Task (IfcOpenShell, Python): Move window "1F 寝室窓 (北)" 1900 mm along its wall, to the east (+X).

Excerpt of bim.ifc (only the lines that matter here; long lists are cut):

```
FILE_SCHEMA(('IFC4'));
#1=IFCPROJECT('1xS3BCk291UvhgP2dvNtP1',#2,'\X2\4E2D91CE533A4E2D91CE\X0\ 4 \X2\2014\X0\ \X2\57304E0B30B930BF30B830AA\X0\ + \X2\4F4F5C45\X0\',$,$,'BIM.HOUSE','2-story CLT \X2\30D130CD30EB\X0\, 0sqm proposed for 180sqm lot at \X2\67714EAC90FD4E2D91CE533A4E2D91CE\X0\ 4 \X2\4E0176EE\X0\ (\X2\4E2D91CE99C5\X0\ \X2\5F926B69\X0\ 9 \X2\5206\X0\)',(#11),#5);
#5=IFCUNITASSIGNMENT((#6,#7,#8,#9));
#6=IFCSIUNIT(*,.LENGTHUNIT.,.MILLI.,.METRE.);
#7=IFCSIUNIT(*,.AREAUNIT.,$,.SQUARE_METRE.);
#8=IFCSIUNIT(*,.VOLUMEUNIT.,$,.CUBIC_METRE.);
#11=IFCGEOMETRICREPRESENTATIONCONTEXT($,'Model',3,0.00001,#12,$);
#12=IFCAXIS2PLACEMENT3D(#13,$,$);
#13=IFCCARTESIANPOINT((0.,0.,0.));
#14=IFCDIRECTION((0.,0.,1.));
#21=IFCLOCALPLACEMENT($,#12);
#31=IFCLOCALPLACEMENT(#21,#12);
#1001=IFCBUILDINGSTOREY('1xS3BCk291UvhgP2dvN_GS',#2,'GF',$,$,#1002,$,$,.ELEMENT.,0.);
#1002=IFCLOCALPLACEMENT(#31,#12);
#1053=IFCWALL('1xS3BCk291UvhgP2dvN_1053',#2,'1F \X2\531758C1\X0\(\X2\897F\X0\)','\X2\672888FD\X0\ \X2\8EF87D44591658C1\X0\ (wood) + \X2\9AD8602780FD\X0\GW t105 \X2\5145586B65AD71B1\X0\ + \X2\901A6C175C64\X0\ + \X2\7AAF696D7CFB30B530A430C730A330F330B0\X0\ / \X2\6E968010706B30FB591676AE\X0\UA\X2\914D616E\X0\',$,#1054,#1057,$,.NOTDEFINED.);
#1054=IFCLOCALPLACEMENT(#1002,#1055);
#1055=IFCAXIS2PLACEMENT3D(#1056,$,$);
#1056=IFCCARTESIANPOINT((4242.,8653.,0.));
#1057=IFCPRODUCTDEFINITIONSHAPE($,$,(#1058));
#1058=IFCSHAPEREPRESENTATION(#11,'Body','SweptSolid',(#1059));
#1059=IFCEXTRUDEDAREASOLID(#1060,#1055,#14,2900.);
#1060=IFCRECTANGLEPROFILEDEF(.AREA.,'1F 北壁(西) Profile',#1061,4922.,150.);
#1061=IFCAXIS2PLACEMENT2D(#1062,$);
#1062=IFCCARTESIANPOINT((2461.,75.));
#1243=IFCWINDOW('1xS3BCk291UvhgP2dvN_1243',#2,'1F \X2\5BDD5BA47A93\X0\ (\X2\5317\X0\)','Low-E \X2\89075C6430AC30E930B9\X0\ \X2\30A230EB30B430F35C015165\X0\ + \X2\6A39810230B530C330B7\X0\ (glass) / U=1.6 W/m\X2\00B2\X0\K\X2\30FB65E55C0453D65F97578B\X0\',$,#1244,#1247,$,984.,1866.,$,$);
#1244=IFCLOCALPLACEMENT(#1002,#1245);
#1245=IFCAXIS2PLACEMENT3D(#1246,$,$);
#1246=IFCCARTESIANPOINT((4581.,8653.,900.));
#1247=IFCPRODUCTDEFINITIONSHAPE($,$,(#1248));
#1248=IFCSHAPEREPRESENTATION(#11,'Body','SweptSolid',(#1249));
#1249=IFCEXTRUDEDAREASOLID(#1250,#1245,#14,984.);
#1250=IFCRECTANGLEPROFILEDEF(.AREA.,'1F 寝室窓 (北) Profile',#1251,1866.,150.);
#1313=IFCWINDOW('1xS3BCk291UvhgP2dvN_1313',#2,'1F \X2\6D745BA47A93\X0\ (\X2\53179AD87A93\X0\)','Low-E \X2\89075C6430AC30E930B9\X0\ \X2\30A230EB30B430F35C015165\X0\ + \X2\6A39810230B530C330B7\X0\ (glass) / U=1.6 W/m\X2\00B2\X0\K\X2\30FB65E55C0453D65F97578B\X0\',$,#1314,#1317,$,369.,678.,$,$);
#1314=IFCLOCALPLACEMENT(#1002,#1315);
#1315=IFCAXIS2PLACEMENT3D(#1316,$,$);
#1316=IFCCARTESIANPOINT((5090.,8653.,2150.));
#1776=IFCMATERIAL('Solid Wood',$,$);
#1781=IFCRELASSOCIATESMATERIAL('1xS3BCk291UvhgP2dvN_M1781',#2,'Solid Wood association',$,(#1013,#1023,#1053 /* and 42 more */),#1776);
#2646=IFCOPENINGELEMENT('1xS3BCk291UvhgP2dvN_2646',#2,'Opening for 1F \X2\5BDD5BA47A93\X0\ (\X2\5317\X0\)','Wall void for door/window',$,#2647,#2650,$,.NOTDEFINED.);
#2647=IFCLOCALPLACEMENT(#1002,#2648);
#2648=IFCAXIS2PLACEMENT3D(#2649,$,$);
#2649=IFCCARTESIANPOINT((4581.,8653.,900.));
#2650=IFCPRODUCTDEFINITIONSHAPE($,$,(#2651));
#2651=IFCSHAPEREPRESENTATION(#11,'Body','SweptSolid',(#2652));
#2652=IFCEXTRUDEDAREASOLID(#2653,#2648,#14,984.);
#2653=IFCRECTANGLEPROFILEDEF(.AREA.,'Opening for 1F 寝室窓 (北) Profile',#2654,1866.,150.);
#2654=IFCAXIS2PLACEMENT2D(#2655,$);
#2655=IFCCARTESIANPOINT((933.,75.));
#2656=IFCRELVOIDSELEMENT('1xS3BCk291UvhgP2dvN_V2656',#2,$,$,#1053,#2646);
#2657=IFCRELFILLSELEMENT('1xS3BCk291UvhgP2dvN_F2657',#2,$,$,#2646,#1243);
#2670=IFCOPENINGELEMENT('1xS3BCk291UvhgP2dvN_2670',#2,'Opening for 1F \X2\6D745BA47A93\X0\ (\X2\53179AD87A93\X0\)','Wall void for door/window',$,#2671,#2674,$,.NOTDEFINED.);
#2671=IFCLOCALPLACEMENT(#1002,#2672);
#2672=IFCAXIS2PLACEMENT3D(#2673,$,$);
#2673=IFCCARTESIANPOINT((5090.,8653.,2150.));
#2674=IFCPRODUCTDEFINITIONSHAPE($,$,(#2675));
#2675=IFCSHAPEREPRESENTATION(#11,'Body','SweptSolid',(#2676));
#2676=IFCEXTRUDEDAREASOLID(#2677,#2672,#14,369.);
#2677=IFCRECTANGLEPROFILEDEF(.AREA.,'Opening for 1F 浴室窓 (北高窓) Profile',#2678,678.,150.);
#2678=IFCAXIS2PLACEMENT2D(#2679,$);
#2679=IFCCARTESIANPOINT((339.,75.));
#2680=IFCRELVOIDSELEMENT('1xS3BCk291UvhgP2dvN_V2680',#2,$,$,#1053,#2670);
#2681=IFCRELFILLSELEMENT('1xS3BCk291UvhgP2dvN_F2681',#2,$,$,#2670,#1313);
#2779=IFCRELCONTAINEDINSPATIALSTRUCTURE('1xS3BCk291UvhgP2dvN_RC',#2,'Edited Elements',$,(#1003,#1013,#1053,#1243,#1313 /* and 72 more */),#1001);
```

```python
import ifcopenshell
import ifcopenshell.api.geometry
import ifcopenshell.util.placement

model = ifcopenshell.open("bim.ifc")

window = model.by_id(1243)
opening = window.FillsVoids[0].RelatingOpeningElement
wall = opening.VoidsElements[0].RelatingBuildingElement

wall_matrix = ifcopenshell.util.placement.get_local_placement(wall.ObjectPlacement)
shift = wall_matrix[:3, 0] * 1900.0
before = ifcopenshell.util.placement.get_local_placement(window.ObjectPlacement)[:3, 3].copy()

# The window is not placed relative to its opening, so move both.
for product in (opening, window):
    matrix = ifcopenshell.util.placement.get_local_placement(product.ObjectPlacement)
    matrix[:3, 3] += shift
    ifcopenshell.api.geometry.edit_object_placement(model, product=product, matrix=matrix, is_si=False)

after = ifcopenshell.util.placement.get_local_placement(window.ObjectPlacement)[:3, 3]
print("window moved by", (after - before).round(3) + 0.0)

model.write("bim-out.ifc")
```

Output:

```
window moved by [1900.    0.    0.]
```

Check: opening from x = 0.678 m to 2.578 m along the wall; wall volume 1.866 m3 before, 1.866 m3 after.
